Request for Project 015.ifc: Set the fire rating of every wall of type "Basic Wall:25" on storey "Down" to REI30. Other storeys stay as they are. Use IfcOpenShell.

First a look at what the model holds.

```python
import ifcopenshell
import ifcopenshell.util.element

model = ifcopenshell.open("Project 015.ifc")
print(model.schema)
storey = next(s for s in model.by_type("IfcBuildingStorey") if s.Name == "Down")
walls = [e for e in ifcopenshell.util.element.get_decomposition(storey) if e.is_a("IfcWall")]
seen = {}
for e in walls:
    element_type = ifcopenshell.util.element.get_type(e)
    key = (element_type.Name if element_type != e and element_type else None, ifcopenshell.util.element.get_pset(e, "Pset_WallCommon", "FireRating"))
    seen[key] = seen.get(key, 0) + 1
for (name, value), count in sorted(seen.items(), key=str):
    print(count, "x", name, "|", value)
```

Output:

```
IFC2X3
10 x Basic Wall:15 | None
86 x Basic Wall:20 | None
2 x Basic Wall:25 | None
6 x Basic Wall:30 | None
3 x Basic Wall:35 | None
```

```python
import ifcopenshell
import ifcopenshell.api.pset
import ifcopenshell.util.element

model = ifcopenshell.open("Project 015.ifc")

storey = next(s for s in model.by_type("IfcBuildingStorey") if s.Name == "Down")
walls = [e for e in ifcopenshell.util.element.get_decomposition(storey) if e.is_a("IfcWall")]

count = 0
for e in walls:
    element_type = ifcopenshell.util.element.get_type(e)
    if element_type in (None, e) or element_type.Name != "Basic Wall:25":
        continue
    # add_pset returns the element's existing set when there is one.
    pset = ifcopenshell.api.pset.add_pset(model, product=e, name="Pset_WallCommon")
    ifcopenshell.api.pset.edit_pset(model, pset=pset, properties={"FireRating": "REI30"})
    count += 1

print(count, "walls updated")

model.write("Project 015_edited.ifc")
```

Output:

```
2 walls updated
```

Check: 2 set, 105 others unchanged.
